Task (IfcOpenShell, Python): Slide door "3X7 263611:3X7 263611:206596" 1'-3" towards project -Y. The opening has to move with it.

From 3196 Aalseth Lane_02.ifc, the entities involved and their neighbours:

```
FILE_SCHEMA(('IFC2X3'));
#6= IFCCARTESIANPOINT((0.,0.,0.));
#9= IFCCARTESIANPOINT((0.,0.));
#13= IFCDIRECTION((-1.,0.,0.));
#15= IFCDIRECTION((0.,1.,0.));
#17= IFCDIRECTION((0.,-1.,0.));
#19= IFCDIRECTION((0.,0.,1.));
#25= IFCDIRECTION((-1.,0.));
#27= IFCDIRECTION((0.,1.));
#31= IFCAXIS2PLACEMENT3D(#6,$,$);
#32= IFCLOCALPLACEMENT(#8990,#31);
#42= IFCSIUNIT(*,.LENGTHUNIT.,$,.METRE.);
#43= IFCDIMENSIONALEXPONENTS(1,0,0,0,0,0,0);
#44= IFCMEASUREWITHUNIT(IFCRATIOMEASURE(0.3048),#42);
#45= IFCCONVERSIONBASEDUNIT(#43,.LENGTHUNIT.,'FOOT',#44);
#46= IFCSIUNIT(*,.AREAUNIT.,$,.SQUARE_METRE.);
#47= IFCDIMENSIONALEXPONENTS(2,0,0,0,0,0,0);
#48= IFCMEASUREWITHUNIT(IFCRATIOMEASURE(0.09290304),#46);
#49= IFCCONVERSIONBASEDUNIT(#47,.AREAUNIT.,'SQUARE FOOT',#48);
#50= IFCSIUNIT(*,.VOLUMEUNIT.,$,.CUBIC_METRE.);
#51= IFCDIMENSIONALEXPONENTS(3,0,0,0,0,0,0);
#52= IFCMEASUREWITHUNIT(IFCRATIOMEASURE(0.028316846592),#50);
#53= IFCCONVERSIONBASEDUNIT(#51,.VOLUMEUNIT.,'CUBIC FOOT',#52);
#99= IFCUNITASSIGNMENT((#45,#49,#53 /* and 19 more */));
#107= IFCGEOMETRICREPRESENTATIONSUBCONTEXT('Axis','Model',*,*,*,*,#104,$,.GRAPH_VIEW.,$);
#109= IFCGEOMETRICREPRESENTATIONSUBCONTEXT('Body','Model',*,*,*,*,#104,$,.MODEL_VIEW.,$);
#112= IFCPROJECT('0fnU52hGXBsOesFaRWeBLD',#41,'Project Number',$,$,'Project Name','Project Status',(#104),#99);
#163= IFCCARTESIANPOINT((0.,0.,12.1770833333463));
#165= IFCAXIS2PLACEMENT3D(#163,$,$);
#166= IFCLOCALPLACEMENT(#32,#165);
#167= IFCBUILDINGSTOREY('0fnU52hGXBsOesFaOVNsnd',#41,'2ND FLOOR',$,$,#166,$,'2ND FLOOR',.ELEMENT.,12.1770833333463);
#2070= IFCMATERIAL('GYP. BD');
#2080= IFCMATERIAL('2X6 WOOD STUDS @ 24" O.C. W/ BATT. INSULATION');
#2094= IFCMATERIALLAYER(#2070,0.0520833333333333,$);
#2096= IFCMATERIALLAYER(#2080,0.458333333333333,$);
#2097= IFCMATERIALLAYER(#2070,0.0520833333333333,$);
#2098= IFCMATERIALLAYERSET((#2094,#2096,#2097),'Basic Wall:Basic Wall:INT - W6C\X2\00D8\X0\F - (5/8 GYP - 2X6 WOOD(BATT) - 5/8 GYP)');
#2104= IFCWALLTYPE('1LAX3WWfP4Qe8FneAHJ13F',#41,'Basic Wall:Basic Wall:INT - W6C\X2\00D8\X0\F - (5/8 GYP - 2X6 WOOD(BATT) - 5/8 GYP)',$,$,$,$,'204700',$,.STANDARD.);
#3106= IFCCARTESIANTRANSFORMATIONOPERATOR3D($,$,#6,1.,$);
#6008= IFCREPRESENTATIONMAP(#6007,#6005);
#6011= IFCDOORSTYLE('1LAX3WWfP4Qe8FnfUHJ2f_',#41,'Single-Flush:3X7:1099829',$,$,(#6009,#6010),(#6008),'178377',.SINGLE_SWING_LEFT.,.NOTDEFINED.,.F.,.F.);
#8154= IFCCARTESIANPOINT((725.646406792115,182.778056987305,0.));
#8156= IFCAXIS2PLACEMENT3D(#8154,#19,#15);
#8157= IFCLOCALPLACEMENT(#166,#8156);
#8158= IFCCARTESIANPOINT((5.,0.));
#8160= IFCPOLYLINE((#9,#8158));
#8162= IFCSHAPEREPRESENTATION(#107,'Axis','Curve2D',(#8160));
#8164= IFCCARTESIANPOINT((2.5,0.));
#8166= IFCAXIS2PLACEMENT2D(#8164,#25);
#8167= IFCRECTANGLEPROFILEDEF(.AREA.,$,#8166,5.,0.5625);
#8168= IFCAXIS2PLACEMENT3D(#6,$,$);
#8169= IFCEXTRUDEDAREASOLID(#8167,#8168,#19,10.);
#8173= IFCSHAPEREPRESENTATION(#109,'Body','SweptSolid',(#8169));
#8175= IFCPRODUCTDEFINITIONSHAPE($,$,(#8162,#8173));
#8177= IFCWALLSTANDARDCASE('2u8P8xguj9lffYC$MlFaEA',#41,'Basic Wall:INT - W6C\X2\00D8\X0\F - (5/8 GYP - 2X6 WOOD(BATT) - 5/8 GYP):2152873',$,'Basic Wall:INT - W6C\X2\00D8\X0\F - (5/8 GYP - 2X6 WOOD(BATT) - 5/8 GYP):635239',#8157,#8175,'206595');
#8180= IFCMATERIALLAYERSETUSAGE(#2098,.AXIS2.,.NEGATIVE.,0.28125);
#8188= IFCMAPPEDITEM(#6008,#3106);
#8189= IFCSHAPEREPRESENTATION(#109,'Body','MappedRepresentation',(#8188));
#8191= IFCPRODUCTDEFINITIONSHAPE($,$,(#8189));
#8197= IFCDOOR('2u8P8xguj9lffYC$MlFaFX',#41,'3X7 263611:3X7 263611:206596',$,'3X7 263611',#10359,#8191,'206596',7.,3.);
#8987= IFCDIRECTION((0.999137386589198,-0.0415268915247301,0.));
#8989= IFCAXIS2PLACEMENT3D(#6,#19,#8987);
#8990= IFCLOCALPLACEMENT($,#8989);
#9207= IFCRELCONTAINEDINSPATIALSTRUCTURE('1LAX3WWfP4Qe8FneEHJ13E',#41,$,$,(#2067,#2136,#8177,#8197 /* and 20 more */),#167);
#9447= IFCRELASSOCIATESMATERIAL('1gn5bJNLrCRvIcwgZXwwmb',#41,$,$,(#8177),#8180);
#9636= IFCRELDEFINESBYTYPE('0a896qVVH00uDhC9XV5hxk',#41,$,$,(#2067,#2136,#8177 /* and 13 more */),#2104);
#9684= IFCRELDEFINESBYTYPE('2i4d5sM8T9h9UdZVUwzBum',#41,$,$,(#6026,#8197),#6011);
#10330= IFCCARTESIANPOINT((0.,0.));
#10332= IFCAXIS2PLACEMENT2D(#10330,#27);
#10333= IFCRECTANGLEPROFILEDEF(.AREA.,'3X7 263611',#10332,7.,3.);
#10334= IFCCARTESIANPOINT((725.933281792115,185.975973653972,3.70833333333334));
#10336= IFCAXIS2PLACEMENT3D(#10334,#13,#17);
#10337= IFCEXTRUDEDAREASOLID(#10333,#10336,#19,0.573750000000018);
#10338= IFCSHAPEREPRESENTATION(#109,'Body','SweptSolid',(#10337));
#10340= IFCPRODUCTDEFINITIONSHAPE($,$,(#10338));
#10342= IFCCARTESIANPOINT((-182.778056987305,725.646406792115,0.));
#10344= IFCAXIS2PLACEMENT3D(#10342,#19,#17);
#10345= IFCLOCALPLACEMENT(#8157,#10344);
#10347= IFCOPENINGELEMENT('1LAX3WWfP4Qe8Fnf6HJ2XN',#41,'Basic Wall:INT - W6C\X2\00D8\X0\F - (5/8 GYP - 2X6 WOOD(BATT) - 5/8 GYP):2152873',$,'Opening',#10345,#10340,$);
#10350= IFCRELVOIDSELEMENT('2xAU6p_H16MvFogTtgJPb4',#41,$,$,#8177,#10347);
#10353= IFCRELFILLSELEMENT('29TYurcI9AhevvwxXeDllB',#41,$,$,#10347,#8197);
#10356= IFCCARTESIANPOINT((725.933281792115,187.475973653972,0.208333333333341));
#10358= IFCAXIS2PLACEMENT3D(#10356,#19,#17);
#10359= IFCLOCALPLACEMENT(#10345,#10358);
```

```python
import ifcopenshell
import ifcopenshell.api.geometry
import ifcopenshell.util.placement
import ifcopenshell.util.unit

model = ifcopenshell.open("3196 Aalseth Lane_02.ifc")
unit_scale = ifcopenshell.util.unit.calculate_unit_scale(model)

door = model.by_guid("2u8P8xguj9lffYC$MlFaFX")
opening = door.FillsVoids[0].RelatingOpeningElement
wall = opening.VoidsElements[0].RelatingBuildingElement

wall_matrix = ifcopenshell.util.placement.get_local_placement(wall.ObjectPlacement)
shift = wall_matrix[:3, 0] * -15 * 0.0254 / unit_scale
before = ifcopenshell.util.placement.get_local_placement(door.ObjectPlacement)[:3, 3].copy()

# The door is placed relative to its opening, so it follows when the opening moves.
matrix = ifcopenshell.util.placement.get_local_placement(opening.ObjectPlacement)
matrix[:3, 3] += shift
ifcopenshell.api.geometry.edit_object_placement(
    model, product=opening, matrix=matrix, is_si=False, should_transform_children=True
)

after = ifcopenshell.util.placement.get_local_placement(door.ObjectPlacement)[:3, 3]
print("door moved by", (after - before).round(3) + 0.0)

model.write("3196 Aalseth Lane_02_rev.ifc")
```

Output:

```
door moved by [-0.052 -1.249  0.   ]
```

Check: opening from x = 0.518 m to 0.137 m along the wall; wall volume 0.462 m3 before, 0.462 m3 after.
